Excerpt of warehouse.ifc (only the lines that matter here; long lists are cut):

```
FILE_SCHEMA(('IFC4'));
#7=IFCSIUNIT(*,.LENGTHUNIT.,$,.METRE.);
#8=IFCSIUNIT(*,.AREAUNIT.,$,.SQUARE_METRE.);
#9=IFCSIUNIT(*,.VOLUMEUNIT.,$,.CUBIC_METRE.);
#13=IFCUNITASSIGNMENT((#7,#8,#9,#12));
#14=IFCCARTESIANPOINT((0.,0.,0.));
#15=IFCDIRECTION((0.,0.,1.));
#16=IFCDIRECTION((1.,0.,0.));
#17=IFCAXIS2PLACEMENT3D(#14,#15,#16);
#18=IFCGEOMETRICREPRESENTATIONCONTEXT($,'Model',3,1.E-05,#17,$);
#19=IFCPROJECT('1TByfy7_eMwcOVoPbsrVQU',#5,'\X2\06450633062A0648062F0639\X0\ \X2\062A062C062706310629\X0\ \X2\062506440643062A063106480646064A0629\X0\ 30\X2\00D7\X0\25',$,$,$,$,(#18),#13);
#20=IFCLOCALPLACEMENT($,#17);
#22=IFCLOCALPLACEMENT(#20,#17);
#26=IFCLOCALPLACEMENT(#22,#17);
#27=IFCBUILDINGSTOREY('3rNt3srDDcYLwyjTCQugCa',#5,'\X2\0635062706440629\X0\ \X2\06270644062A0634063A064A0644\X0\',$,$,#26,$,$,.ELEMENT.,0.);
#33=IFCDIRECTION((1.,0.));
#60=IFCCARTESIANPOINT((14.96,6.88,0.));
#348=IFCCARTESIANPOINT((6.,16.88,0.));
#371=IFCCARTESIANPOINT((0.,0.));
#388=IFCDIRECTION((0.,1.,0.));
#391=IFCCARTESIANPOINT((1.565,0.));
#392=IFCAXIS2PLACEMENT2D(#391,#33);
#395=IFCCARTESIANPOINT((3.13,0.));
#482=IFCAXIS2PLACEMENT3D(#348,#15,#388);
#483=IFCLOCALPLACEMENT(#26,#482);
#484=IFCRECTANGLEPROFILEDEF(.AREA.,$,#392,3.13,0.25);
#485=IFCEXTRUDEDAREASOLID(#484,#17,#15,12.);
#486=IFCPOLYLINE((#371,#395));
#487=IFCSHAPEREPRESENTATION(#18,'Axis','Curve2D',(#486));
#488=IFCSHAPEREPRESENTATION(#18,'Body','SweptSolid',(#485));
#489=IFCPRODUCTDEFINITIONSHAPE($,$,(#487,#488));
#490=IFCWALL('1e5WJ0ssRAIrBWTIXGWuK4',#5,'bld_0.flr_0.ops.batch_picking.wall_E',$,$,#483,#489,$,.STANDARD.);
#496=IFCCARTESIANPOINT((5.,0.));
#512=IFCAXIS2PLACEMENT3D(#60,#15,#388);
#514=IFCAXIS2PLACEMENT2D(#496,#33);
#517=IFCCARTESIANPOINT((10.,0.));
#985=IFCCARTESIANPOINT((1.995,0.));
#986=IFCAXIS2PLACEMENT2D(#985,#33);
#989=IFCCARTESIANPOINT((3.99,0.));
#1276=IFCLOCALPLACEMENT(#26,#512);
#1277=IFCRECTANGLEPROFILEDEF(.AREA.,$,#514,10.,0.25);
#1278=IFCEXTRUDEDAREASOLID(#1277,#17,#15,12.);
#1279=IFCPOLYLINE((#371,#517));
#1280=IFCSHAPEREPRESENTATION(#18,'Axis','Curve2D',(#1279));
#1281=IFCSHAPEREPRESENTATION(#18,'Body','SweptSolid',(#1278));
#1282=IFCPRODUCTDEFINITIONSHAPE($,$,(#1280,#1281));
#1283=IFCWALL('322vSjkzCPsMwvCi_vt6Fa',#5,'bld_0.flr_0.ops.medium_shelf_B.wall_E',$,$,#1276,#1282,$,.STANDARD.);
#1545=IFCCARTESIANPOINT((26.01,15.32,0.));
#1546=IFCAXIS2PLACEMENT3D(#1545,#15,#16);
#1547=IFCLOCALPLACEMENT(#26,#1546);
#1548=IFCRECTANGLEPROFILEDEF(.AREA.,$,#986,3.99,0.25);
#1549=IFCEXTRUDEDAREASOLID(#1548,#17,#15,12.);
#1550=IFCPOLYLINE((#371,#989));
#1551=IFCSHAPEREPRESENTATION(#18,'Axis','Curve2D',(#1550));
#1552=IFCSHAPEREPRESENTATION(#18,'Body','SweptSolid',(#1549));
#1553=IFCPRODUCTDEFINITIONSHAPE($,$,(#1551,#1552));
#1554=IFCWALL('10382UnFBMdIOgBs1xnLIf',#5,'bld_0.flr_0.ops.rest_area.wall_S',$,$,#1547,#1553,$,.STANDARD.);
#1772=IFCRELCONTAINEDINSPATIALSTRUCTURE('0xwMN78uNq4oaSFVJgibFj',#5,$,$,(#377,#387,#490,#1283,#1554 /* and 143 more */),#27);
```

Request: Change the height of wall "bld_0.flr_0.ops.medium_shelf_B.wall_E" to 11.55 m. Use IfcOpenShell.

```python
import ifcopenshell
import ifcopenshell.geom
import ifcopenshell.util.shape
import ifcopenshell.util.unit

model = ifcopenshell.open("warehouse.ifc")
unit_scale = ifcopenshell.util.unit.calculate_unit_scale(model)
settings = ifcopenshell.geom.settings()


def volume(element):
    """Net volume in cubic metres, openings subtracted."""
    shape = ifcopenshell.geom.create_shape(settings, element)
    return ifcopenshell.util.shape.get_volume(shape.geometry)


wall = model.by_guid("322vSjkzCPsMwvCi_vt6Fa")
before = volume(wall)

body = next(r for r in wall.Representation.Representations if r.RepresentationIdentifier == "Body")
solid = body.Items[0]
old_height = solid.Depth
solid.Depth = 11.55 / unit_scale
after = volume(wall)

print(f"height {old_height:g} -> {solid.Depth:g}, volume {before:.3f} -> {after:.3f} m3")

model.write("warehouse_updated.ifc")
```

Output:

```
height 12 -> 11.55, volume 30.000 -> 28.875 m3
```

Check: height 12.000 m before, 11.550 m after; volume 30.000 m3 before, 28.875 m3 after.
